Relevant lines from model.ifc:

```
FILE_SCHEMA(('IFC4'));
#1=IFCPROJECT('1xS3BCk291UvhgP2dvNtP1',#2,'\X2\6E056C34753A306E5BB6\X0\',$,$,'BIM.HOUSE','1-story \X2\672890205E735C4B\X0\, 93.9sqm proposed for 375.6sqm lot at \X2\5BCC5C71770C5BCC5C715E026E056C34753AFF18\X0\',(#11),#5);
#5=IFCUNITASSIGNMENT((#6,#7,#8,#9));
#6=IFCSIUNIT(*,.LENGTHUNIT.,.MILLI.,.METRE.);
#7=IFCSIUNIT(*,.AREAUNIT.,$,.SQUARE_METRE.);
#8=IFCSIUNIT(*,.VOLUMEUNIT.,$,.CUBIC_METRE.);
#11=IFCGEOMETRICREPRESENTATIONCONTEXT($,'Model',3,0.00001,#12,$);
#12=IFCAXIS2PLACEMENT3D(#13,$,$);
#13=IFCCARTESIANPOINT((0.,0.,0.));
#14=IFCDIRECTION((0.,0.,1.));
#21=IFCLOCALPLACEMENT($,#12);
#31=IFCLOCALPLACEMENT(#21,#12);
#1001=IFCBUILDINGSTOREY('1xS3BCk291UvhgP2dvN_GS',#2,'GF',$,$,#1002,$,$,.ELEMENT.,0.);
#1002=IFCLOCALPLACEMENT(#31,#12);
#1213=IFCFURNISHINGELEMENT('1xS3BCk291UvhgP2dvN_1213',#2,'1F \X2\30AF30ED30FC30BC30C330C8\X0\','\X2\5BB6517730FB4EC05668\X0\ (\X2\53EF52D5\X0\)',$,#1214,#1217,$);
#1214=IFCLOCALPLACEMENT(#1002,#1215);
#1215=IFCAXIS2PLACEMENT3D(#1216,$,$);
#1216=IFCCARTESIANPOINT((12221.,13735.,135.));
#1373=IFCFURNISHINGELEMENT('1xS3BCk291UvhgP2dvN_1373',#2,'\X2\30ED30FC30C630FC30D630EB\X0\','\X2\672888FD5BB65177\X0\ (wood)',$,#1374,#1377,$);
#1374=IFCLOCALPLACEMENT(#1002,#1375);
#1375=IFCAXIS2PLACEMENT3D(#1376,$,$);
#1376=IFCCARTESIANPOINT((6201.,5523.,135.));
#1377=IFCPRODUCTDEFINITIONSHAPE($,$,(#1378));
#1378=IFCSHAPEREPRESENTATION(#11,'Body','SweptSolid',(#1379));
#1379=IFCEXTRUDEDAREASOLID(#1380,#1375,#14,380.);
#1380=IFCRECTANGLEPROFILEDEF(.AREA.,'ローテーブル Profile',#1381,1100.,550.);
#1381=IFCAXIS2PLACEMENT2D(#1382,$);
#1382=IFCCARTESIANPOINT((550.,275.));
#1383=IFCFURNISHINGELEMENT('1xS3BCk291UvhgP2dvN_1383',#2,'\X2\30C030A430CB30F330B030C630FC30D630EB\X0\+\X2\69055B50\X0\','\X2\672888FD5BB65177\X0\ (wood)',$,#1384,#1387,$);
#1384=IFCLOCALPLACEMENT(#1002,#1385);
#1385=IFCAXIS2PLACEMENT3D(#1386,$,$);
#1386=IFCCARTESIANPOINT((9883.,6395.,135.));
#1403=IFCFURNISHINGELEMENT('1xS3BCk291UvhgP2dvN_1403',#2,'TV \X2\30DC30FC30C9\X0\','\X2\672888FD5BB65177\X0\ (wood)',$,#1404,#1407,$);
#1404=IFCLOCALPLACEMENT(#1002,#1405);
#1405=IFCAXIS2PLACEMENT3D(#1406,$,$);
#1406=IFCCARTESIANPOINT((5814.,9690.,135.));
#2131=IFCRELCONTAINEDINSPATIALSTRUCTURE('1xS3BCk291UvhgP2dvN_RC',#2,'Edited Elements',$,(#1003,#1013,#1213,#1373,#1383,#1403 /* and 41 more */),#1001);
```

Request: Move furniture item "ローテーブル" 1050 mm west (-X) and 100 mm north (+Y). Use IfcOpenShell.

```python
import ifcopenshell
import ifcopenshell.api.geometry
import ifcopenshell.util.placement
import ifcopenshell.util.unit

model = ifcopenshell.open("model.ifc")
unit_scale = ifcopenshell.util.unit.calculate_unit_scale(model)

item = model.by_guid("1xS3BCk291UvhgP2dvN_1373")
matrix = ifcopenshell.util.placement.get_local_placement(item.ObjectPlacement)
matrix[0, 3] -= 1.05 / unit_scale
matrix[1, 3] += 0.1 / unit_scale
ifcopenshell.api.geometry.edit_object_placement(model, product=item, matrix=matrix, is_si=False)

print(ifcopenshell.util.placement.get_local_placement(item.ObjectPlacement).round(3) + 0.0)

model.write("model_v2.ifc")
```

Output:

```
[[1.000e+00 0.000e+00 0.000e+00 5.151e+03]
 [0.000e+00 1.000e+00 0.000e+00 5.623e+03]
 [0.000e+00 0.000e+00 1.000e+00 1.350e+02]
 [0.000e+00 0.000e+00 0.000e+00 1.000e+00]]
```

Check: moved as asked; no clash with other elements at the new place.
